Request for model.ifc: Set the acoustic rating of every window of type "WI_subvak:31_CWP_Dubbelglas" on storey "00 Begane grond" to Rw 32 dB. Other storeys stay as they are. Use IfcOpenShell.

First a look at what the model holds.

```python
import ifcopenshell
import ifcopenshell.util.element

model = ifcopenshell.open("model.ifc")
print(model.schema)
storey = next(s for s in model.by_type("IfcBuildingStorey") if s.Name == "00 Begane grond")
windows = [e for e in ifcopenshell.util.element.get_decomposition(storey) if e.is_a("IfcWindow")]
seen = {}
for e in windows:
    element_type = ifcopenshell.util.element.get_type(e)
    key = (element_type.Name if element_type != e and element_type else None, ifcopenshell.util.element.get_pset(e, "Pset_WindowCommon", "AcousticRating"))
    seen[key] = seen.get(key, 0) + 1
for (name, value), count in sorted(seen.items(), key=str):
    print(count, "x", name, "|", value)
```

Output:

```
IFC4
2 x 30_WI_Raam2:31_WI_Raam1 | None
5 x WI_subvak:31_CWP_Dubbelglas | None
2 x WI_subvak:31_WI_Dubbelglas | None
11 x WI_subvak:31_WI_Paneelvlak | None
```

```python
import ifcopenshell
import ifcopenshell.api.pset
import ifcopenshell.util.element

model = ifcopenshell.open("model.ifc")

storey = next(s for s in model.by_type("IfcBuildingStorey") if s.Name == "00 Begane grond")
windows = [e for e in ifcopenshell.util.element.get_decomposition(storey) if e.is_a("IfcWindow")]

count = 0
for e in windows:
    element_type = ifcopenshell.util.element.get_type(e)
    if element_type in (None, e) or element_type.Name != "WI_subvak:31_CWP_Dubbelglas":
        continue
    # add_pset returns the element's existing set when there is one.
    pset = ifcopenshell.api.pset.add_pset(model, product=e, name="Pset_WindowCommon")
    ifcopenshell.api.pset.edit_pset(model, pset=pset, properties={"AcousticRating": "Rw 32 dB"})
    count += 1

print(count, "windows updated")

model.write("model_rev.ifc")
```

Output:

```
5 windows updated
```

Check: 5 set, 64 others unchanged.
